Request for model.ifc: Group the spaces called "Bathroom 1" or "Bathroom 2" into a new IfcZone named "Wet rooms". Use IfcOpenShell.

First a look at what the model holds.

```python
import ifcopenshell

model = ifcopenshell.open("model.ifc")
print(model.schema)
seen = {}
for space in model.by_type("IfcSpace"):
    seen[space.LongName] = seen.get(space.LongName, 0) + 1
for name, count in sorted(seen.items(), key=str):
    print(count, "x", name)
print("zones:", [z.Name for z in model.by_type("IfcZone")][:20])
```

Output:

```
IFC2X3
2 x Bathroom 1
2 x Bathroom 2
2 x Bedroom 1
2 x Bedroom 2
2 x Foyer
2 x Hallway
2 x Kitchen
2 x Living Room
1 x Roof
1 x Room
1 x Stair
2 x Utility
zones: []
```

```python
import ifcopenshell
import ifcopenshell.api.group
import ifcopenshell.api.root

model = ifcopenshell.open("model.ifc")

names = {"Bathroom 1", "Bathroom 2"}
spaces = [s for s in model.by_type("IfcSpace") if s.LongName in names]

zone = ifcopenshell.api.root.create_entity(model, ifc_class="IfcZone", name="Wet rooms")
ifcopenshell.api.group.assign_group(model, products=spaces, group=zone)
print(len(spaces), "spaces in", zone.Name)

model.write("model_updated.ifc")
```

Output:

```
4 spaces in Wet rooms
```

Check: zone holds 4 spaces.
